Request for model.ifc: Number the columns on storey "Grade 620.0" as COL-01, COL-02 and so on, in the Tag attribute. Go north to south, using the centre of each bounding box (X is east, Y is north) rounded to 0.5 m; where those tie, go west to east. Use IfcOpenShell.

First a look at what the model holds.

```python
import ifcopenshell
import ifcopenshell.util.element
import ifcopenshell.util.placement

model = ifcopenshell.open("model.ifc")
print(model.schema)
storey = next(s for s in model.by_type("IfcBuildingStorey") if s.Name == "Grade 620.0")
columns = [e for e in ifcopenshell.util.element.get_decomposition(storey) if e.is_a("IfcColumn")]
for e in sorted(columns, key=lambda e: e.id()):
    origin = ifcopenshell.util.placement.get_local_placement(e.ObjectPlacement)[:3, 3]
    print(e.id(), e.Tag, e.Name, origin.round(2) + 0.0, sep=" | ")
```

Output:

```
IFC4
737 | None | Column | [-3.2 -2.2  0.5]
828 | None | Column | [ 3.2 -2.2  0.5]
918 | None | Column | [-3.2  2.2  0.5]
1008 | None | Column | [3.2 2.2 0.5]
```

```python
import ifcopenshell
import ifcopenshell.geom
import ifcopenshell.util.element
import ifcopenshell.util.shape

model = ifcopenshell.open("model.ifc")
settings = ifcopenshell.geom.settings()
settings.set("use-world-coords", True)


def centre(element):
    shape = ifcopenshell.geom.create_shape(settings, element)
    return ifcopenshell.util.shape.get_bbox_centroid(shape.geometry)


storey = next(s for s in model.by_type("IfcBuildingStorey") if s.Name == "Grade 620.0")
columns = [e for e in ifcopenshell.util.element.get_decomposition(storey) if e.is_a("IfcColumn")]

# Insertion points can sit at a corner or the storey origin, so sort by the geometry (in metres).
centres = {e: centre(e) for e in columns}
columns.sort(key=lambda e: (-round(centres[e][1] / 0.5), centres[e][0]))

for i, e in enumerate(columns, start=1):
    number = f"COL-{i:02d}"
    e.Tag = number
    print(e.id(), number)

model.write("model_v2.ifc")
```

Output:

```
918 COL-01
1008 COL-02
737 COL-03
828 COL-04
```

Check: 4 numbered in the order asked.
